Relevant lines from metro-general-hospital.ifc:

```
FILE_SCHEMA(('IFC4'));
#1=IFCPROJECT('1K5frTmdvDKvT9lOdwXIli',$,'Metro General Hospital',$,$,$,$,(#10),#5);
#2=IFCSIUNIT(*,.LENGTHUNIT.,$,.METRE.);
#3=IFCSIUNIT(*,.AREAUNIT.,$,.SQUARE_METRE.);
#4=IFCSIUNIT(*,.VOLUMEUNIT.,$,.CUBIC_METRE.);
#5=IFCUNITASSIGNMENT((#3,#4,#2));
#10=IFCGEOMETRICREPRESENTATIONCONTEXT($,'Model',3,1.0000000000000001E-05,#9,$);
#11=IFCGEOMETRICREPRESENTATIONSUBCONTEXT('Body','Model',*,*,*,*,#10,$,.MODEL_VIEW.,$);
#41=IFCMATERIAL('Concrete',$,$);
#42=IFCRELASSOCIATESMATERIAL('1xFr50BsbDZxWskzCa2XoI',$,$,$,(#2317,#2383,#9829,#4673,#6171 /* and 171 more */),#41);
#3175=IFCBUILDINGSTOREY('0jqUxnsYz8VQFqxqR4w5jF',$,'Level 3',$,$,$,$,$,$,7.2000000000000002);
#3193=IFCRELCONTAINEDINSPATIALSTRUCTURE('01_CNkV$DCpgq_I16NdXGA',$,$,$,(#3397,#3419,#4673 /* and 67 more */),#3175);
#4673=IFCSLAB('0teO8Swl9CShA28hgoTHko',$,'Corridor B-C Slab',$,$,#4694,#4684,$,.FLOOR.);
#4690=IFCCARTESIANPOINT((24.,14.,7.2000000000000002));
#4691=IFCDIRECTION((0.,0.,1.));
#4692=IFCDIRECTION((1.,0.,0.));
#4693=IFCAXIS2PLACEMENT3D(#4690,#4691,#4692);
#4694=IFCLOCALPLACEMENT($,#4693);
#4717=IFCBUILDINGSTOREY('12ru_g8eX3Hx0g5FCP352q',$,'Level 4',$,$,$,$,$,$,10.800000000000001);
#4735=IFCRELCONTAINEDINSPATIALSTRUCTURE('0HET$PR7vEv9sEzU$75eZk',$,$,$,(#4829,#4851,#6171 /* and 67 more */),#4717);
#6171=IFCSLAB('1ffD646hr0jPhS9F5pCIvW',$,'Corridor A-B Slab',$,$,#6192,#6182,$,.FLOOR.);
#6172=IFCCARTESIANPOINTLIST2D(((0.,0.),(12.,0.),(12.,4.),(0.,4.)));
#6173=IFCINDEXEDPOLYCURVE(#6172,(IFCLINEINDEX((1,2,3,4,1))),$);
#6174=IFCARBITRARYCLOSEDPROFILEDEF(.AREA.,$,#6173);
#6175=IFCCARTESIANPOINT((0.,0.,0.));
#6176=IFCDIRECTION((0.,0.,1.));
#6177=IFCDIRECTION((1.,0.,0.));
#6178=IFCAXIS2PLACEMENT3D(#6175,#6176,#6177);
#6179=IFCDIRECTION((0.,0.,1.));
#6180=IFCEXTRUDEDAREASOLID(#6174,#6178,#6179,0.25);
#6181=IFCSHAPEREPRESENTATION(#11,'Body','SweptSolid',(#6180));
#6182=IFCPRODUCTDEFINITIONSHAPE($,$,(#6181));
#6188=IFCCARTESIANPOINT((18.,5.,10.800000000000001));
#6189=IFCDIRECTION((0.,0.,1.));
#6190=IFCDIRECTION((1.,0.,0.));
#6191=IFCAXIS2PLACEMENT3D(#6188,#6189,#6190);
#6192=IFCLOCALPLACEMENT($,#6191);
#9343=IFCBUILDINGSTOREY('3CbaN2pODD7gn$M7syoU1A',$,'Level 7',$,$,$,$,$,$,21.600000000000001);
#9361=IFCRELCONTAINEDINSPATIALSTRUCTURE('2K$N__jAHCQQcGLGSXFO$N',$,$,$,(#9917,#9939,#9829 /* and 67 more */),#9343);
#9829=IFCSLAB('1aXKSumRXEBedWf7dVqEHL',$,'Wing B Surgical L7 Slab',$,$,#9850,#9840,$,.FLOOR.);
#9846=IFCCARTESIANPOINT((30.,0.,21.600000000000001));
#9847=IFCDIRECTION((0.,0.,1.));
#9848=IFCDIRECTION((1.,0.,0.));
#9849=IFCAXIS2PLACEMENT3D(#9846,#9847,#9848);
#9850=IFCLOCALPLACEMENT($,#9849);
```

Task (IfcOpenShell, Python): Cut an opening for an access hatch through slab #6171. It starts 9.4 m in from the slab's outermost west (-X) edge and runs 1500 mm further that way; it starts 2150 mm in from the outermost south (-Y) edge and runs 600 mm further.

```python
import numpy as np
import ifcopenshell
import ifcopenshell.api.feature
import ifcopenshell.api.geometry
import ifcopenshell.api.root
import ifcopenshell.geom
import ifcopenshell.util.placement
import ifcopenshell.util.representation
import ifcopenshell.util.shape
import ifcopenshell.util.unit

model = ifcopenshell.open("metro-general-hospital.ifc")
unit_scale = ifcopenshell.util.unit.calculate_unit_scale(model)
settings = ifcopenshell.geom.settings()


def volume(element):
    """Net volume in cubic metres, openings subtracted."""
    shape = ifcopenshell.geom.create_shape(settings, element)
    return ifcopenshell.util.shape.get_volume(shape.geometry)


slab = model.by_guid("1ffD646hr0jPhS9F5pCIvW")
before = volume(slab)

# Extent in the slab's own axes, in metres. The edges named are its -X and -Y sides.
slab_shape = ifcopenshell.geom.create_shape(settings, slab)
vertices = ifcopenshell.util.shape.get_vertices(slab_shape.geometry)
x_min, y_min, bottom = vertices.min(axis=0)
top = vertices[:, 2].max()

opening = ifcopenshell.api.root.create_entity(model, ifc_class="IfcOpeningElement", name="Access hatch opening", predefined_type="OPENING")
context = ifcopenshell.util.representation.get_context(model, "Model", "Body", "MODEL_VIEW")
width, depth = 1.5, 0.6
outline = [(0.0, 0.0), (width, 0.0), (width, depth), (0.0, depth), (0.0, 0.0)]
# Overshoot both faces by 50 mm so the cut is clean.
shape = ifcopenshell.api.geometry.add_slab_representation(
    model, context=context, depth=top - bottom + 0.1, polyline=outline
)
ifcopenshell.api.geometry.assign_representation(model, product=opening, representation=shape)

matrix = ifcopenshell.util.placement.get_local_placement(slab.ObjectPlacement)
matrix[:, 3] = matrix @ np.append(np.array([x_min + 9.4, y_min + 2.15, bottom - 0.05]) / unit_scale, 1.0)
ifcopenshell.api.geometry.edit_object_placement(model, product=opening, matrix=matrix, is_si=False)
ifcopenshell.api.feature.add_feature(model, feature=opening, element=slab)

after = volume(slab)

print(f"slab volume {before:.3f} -> {after:.3f} m3")

model.write("metro-general-hospital_edited.ifc")
```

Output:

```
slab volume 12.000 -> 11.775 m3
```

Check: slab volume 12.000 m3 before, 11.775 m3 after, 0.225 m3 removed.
